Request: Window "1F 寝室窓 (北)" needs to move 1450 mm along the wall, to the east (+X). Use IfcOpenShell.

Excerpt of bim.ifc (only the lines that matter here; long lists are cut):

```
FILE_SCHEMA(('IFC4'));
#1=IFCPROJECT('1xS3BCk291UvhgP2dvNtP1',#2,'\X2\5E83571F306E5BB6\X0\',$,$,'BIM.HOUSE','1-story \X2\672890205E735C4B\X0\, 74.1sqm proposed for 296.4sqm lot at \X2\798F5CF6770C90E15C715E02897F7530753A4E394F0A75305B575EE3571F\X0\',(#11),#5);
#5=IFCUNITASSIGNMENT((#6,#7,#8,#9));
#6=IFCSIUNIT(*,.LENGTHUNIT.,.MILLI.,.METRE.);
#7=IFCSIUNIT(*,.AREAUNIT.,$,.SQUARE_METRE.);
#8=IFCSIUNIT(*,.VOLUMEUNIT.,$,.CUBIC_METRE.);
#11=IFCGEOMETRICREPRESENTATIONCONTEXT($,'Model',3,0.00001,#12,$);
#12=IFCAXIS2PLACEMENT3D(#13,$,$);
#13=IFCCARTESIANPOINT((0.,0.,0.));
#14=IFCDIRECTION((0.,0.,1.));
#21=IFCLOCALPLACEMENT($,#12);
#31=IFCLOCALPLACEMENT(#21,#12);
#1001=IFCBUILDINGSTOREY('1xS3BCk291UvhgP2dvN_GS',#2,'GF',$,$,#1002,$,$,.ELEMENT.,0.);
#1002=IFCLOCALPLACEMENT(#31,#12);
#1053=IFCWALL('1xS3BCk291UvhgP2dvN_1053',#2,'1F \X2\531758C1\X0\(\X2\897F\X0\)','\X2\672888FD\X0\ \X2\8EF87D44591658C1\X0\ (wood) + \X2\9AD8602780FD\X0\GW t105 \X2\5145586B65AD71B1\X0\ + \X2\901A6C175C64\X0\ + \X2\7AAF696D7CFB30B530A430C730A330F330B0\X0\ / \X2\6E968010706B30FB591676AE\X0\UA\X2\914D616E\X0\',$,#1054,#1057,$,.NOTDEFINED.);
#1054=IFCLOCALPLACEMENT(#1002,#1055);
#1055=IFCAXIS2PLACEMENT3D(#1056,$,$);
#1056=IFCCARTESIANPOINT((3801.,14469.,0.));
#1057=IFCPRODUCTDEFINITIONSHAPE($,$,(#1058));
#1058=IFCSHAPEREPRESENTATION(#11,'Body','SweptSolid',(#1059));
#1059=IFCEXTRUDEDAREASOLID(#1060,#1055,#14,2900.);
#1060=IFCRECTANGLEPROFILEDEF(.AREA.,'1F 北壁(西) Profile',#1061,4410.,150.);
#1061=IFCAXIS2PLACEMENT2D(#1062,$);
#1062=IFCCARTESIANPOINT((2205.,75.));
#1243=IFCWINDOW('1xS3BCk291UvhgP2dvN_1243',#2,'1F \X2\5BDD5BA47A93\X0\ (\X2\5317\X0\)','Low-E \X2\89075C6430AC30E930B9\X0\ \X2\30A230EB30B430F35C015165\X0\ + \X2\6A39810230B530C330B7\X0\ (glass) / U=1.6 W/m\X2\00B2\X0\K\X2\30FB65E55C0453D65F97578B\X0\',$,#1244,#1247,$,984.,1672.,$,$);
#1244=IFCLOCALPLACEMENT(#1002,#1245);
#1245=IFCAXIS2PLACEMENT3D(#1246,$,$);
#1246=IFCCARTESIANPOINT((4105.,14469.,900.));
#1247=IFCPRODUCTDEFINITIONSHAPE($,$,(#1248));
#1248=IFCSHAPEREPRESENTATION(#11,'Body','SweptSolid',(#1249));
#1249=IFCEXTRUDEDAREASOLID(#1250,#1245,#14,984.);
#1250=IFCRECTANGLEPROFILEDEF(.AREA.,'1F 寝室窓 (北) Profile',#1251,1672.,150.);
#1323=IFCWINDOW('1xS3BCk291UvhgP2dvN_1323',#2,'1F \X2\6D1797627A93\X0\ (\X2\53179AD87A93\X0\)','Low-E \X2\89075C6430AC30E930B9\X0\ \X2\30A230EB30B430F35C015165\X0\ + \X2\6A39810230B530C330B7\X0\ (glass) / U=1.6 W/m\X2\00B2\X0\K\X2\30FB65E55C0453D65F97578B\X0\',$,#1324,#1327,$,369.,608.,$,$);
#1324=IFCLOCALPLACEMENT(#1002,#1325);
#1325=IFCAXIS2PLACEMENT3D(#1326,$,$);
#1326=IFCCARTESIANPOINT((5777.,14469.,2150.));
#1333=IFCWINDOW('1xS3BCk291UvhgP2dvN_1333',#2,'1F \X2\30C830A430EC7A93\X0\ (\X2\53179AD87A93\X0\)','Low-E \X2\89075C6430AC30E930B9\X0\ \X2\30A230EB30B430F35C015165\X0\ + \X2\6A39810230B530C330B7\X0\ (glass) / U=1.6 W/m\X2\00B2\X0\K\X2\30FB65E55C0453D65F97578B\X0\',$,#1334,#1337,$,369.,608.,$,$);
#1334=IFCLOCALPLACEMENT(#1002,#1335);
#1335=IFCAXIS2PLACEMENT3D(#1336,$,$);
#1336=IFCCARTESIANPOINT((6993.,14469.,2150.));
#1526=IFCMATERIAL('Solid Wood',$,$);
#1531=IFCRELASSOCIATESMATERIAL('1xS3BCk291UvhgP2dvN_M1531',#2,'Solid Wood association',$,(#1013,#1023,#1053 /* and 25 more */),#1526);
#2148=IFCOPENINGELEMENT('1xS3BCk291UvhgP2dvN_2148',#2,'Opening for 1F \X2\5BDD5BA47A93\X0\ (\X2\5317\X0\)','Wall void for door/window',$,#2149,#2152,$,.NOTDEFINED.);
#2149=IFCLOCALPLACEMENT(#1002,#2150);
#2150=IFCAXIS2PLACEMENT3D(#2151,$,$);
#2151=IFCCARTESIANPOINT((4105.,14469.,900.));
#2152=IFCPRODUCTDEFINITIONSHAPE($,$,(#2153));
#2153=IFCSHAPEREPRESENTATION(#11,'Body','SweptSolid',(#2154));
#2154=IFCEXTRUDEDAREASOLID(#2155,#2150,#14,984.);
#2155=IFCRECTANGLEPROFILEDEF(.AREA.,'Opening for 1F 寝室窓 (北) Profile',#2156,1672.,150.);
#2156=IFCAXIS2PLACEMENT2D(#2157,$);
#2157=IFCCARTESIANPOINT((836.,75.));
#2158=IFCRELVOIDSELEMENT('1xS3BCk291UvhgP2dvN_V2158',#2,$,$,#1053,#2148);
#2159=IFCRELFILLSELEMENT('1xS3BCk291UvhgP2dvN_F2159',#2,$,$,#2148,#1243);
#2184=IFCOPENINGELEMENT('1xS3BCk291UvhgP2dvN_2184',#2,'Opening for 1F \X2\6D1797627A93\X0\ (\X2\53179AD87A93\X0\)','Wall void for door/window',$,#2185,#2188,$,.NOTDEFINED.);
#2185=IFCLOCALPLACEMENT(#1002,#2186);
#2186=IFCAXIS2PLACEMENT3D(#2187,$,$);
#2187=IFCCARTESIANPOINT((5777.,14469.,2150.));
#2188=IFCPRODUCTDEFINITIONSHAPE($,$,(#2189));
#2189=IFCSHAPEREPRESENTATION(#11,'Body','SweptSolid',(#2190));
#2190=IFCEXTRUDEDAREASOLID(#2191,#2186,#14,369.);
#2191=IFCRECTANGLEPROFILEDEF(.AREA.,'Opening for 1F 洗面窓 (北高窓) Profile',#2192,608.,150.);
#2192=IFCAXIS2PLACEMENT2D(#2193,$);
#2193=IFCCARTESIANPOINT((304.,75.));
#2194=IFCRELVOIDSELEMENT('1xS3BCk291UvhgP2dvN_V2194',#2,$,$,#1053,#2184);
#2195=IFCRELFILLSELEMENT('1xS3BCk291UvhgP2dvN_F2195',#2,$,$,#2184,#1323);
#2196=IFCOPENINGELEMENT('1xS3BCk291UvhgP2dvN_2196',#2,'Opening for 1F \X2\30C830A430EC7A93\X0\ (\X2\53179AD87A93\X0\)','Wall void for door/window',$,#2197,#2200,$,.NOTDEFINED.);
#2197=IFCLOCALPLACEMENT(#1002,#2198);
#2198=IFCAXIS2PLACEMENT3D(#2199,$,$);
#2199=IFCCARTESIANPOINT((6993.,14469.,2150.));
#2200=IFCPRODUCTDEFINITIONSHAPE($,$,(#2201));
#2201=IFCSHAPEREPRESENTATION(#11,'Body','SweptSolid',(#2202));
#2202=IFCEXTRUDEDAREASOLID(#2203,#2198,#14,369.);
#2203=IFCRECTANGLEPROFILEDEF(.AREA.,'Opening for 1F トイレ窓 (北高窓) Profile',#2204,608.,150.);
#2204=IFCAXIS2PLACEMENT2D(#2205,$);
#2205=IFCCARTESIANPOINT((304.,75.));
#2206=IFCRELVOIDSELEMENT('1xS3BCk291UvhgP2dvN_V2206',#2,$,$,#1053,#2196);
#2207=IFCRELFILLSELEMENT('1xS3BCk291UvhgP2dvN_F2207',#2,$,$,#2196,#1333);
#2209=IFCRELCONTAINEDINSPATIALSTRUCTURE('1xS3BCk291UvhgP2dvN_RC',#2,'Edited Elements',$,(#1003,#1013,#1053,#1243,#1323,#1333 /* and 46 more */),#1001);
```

```python
import ifcopenshell
import ifcopenshell.api.geometry
import ifcopenshell.util.placement

model = ifcopenshell.open("bim.ifc")

window = model.by_guid("1xS3BCk291UvhgP2dvN_1243")
opening = window.FillsVoids[0].RelatingOpeningElement
wall = opening.VoidsElements[0].RelatingBuildingElement

wall_matrix = ifcopenshell.util.placement.get_local_placement(wall.ObjectPlacement)
shift = wall_matrix[:3, 0] * 1450.0
before = ifcopenshell.util.placement.get_local_placement(window.ObjectPlacement)[:3, 3].copy()

# The window is not placed relative to its opening, so move both.
for product in (opening, window):
    matrix = ifcopenshell.util.placement.get_local_placement(product.ObjectPlacement)
    matrix[:3, 3] += shift
    ifcopenshell.api.geometry.edit_object_placement(model, product=product, matrix=matrix, is_si=False)

after = ifcopenshell.util.placement.get_local_placement(window.ObjectPlacement)[:3, 3]
print("window moved by", (after - before).round(3) + 0.0)

model.write("bim-out.ifc")
```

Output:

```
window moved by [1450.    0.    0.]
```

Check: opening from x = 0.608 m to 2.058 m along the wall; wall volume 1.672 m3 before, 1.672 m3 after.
